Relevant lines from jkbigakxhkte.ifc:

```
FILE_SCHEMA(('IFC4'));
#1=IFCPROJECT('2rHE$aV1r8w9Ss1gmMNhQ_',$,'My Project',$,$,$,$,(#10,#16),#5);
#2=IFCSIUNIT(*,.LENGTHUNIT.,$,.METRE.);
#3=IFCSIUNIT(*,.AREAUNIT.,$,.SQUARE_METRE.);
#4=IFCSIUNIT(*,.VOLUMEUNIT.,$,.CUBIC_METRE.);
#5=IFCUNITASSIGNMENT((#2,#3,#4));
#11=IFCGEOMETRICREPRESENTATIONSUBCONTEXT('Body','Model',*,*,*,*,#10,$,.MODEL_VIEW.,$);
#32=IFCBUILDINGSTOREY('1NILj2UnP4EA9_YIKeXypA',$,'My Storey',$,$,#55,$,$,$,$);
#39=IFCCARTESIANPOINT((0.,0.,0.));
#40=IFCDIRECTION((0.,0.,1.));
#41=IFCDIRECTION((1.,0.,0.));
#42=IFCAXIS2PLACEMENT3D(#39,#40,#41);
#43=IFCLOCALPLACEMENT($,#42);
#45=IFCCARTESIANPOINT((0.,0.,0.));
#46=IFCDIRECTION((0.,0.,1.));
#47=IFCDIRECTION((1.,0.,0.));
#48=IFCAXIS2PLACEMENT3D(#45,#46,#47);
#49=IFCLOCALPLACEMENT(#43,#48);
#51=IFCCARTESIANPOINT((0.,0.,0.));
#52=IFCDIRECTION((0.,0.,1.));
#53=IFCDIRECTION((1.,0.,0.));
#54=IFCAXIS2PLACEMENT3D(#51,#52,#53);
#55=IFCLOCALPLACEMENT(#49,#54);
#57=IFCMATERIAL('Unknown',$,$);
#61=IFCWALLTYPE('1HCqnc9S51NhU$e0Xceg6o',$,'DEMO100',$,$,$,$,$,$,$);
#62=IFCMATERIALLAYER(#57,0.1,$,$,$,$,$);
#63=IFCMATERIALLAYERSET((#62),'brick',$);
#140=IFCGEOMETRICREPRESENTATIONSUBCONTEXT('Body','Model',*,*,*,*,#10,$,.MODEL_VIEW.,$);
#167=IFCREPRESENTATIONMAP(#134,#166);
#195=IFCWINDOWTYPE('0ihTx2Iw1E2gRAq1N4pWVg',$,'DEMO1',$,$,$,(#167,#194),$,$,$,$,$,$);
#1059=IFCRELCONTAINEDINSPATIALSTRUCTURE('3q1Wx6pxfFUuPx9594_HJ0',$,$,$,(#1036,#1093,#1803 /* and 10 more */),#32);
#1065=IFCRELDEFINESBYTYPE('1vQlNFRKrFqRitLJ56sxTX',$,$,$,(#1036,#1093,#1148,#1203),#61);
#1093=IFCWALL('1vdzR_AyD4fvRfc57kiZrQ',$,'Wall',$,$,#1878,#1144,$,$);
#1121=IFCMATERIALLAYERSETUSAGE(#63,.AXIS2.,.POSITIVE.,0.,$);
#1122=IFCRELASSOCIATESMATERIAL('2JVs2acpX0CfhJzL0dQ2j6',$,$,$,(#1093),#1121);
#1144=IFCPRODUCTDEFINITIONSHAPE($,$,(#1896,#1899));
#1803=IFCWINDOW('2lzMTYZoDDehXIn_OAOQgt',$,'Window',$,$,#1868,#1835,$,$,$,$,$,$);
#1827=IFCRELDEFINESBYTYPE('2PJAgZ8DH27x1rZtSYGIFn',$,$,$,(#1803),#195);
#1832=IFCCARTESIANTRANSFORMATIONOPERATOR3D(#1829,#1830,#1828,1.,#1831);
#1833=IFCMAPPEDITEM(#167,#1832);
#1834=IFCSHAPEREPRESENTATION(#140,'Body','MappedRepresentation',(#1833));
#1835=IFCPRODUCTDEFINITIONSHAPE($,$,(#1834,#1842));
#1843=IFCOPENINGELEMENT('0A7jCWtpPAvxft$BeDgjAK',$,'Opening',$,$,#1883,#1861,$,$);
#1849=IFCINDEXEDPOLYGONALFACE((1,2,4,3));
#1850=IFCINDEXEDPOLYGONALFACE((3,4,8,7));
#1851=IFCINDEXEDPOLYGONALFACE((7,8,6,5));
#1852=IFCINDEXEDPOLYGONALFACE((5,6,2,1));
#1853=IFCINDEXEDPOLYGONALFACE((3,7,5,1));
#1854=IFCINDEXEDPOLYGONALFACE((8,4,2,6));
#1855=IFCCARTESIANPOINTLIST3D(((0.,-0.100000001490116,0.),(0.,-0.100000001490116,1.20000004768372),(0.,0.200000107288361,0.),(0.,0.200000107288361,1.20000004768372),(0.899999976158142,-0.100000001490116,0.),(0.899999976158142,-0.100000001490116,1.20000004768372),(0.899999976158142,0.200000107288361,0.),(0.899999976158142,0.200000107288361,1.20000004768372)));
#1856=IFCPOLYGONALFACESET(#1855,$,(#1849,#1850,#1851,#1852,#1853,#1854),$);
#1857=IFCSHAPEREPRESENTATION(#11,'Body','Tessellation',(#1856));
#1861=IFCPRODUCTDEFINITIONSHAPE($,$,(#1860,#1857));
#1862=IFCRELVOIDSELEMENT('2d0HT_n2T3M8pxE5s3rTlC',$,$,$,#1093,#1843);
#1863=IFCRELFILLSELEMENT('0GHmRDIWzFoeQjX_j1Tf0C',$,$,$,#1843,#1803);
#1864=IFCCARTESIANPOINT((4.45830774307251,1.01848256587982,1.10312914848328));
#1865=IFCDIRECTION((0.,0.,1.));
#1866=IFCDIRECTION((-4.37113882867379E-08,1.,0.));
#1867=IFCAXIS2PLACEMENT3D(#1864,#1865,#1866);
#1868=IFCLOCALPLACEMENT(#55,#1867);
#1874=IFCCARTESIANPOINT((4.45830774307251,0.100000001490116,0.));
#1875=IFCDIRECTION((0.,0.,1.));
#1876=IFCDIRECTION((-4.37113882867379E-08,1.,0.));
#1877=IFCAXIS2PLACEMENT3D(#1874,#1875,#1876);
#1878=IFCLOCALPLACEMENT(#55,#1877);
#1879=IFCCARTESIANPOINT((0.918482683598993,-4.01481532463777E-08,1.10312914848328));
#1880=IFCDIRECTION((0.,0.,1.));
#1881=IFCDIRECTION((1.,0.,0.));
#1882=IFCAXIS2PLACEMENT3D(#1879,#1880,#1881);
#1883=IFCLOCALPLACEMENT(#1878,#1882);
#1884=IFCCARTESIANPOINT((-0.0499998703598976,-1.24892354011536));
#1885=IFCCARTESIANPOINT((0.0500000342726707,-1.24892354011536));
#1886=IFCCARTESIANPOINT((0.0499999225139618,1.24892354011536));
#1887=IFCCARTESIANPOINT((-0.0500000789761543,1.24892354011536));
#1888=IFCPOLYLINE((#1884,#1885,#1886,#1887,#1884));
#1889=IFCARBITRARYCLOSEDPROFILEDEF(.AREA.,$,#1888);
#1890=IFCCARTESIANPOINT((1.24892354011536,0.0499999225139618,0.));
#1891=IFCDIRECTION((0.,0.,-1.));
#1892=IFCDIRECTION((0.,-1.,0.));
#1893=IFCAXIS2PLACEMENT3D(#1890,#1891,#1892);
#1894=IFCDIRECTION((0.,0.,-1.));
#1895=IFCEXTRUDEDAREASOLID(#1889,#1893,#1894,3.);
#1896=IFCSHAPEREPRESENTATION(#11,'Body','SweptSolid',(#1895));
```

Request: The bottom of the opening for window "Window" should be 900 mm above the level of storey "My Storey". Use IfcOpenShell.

```python
import numpy as np
import ifcopenshell
import ifcopenshell.api.geometry
import ifcopenshell.geom
import ifcopenshell.util.element
import ifcopenshell.util.placement
import ifcopenshell.util.shape
import ifcopenshell.util.unit

model = ifcopenshell.open("jkbigakxhkte.ifc")
unit_scale = ifcopenshell.util.unit.calculate_unit_scale(model)

window = model.by_guid("2lzMTYZoDDehXIn_OAOQgt")
opening = window.FillsVoids[0].RelatingOpeningElement
storey = ifcopenshell.util.element.get_container(window, ifc_class="IfcBuildingStorey")
level = ifcopenshell.util.placement.get_local_placement(storey.ObjectPlacement)[2, 3]

# The opening's origin need not be at the sill, so measure its lowest point.
shape = ifcopenshell.geom.create_shape(ifcopenshell.geom.settings(), opening)
bottom = ifcopenshell.util.shape.get_shape_bottom_elevation(shape, shape.geometry) / unit_scale
dz = level + 0.9 - bottom

shift = np.array([0.0, 0.0, dz])
# The window is not placed relative to its opening, so move both.
for product in (opening, window):
    matrix = ifcopenshell.util.placement.get_local_placement(product.ObjectPlacement)
    matrix[:3, 3] += shift
    ifcopenshell.api.geometry.edit_object_placement(model, product=product, matrix=matrix, is_si=False)

print(f"moved by {dz * unit_scale:+.3f} m")

model.write("jkbigakxhkte_edited.ifc")
```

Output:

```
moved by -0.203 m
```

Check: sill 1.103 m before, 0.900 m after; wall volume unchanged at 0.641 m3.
